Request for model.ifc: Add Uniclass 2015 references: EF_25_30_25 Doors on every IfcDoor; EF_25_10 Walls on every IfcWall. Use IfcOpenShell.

First a look at what the model holds.

```python
import ifcopenshell

model = ifcopenshell.open("model.ifc")
print(model.schema)
print("classifications:", [c.Name for c in model.by_type("IfcClassification")])
for ifc_class in ("IfcDoor", "IfcRoof", "IfcStair", "IfcWall", "IfcWindow"):
    print(ifc_class, len(model.by_type(ifc_class)))
```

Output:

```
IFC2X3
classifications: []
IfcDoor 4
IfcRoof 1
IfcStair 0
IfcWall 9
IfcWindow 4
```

```python
import ifcopenshell
import ifcopenshell.api.classification

model = ifcopenshell.open("model.ifc")

# IFC2X3 requires Source and Edition and has no link from the project to the system.
system = model.create_entity("IfcClassification", Source="NBS", Edition="2015", Name="Uniclass 2015")

codes = {
    "IfcDoor": ("EF_25_30_25", "Doors"),
    "IfcWall": ("EF_25_10", "Walls"),
}
for ifc_class, (code, name) in codes.items():
    products = model.by_type(ifc_class)
    ifcopenshell.api.classification.add_reference(
        model, products=products, classification=system, identification=code, name=name
    )
    print(code, len(products))

model.write("model_rev.ifc")
```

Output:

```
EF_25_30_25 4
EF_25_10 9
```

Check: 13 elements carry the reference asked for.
